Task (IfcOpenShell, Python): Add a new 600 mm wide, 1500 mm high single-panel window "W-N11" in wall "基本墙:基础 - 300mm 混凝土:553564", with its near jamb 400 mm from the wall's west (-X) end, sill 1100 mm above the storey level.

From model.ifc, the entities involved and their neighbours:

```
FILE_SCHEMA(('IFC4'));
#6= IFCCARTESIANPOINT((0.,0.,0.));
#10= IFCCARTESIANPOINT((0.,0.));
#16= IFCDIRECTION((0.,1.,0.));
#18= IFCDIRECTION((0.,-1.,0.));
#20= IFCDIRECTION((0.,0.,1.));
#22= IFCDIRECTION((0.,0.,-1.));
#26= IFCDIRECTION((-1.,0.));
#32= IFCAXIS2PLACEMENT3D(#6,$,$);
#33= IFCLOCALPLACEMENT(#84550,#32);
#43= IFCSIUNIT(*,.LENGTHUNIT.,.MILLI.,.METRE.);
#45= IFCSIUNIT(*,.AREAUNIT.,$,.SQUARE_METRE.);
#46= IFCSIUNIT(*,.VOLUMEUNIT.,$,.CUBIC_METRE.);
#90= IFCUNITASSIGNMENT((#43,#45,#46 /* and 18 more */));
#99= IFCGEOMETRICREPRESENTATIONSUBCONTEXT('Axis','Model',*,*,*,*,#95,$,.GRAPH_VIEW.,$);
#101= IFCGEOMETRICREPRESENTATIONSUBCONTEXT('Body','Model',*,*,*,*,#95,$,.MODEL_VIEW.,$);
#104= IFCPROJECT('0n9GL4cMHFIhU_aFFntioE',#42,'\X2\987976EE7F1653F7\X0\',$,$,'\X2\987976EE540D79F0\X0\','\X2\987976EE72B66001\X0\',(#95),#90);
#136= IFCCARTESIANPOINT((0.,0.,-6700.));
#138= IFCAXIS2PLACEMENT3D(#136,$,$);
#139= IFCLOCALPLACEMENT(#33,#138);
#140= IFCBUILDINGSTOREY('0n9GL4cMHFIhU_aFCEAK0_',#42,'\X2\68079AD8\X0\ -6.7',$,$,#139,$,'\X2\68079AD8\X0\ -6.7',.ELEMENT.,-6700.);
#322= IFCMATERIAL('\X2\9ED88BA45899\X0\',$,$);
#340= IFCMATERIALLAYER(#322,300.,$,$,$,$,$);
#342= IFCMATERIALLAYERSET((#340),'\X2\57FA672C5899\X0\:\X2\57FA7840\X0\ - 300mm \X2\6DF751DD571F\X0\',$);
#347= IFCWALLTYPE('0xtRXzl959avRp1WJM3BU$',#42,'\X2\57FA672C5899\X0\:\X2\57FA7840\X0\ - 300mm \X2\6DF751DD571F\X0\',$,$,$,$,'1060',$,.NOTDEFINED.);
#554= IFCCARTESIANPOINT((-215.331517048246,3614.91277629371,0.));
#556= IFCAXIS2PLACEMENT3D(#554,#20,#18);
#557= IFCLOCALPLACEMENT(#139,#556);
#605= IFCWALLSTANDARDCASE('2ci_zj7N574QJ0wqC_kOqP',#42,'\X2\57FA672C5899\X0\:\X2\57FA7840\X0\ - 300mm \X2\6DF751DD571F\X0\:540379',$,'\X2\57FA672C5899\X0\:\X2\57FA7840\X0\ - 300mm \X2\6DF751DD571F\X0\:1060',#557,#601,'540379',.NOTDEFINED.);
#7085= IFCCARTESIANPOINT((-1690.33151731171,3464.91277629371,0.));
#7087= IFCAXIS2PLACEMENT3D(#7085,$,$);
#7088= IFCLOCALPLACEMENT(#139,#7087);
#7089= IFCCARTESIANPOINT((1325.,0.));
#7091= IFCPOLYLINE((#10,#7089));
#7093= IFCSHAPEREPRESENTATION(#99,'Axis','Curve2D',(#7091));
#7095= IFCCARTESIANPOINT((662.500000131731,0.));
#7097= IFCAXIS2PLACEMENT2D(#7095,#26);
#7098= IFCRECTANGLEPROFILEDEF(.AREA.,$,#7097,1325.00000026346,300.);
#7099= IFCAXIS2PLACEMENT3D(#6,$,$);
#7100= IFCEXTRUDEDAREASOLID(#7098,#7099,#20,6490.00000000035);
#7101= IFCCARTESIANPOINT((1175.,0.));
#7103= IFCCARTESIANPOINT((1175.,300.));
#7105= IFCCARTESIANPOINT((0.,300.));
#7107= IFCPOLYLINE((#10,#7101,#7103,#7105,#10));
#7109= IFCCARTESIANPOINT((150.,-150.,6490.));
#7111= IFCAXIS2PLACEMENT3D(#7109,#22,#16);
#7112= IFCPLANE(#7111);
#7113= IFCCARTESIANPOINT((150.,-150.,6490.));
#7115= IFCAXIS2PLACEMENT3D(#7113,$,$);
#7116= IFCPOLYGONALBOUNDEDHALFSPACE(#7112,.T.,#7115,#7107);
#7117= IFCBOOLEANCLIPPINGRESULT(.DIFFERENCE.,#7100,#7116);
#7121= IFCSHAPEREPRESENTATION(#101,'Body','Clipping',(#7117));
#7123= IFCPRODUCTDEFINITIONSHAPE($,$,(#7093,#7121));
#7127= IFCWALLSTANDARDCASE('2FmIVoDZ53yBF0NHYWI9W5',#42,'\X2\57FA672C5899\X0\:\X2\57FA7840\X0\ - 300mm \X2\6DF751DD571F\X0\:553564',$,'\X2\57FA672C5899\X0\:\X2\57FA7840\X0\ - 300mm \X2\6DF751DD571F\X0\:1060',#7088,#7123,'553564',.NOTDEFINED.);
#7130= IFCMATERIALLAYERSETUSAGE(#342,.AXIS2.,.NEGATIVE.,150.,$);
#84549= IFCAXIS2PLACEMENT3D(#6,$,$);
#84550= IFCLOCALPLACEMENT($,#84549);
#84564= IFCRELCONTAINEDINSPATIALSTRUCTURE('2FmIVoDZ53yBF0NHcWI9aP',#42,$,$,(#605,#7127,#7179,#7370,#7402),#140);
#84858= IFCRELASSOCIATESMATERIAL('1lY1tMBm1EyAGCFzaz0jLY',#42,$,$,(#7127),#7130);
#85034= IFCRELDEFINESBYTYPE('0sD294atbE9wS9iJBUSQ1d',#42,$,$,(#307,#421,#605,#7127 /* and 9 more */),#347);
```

```python
import numpy as np
import ifcopenshell
import ifcopenshell.api.feature
import ifcopenshell.api.geometry
import ifcopenshell.api.root
import ifcopenshell.api.spatial
import ifcopenshell.geom
import ifcopenshell.util.element
import ifcopenshell.util.placement
import ifcopenshell.util.representation
import ifcopenshell.util.shape
import ifcopenshell.util.unit

model = ifcopenshell.open("model.ifc")
unit_scale = ifcopenshell.util.unit.calculate_unit_scale(model)
settings = ifcopenshell.geom.settings()


def volume(element):
    """Net volume in cubic metres, openings subtracted."""
    shape = ifcopenshell.geom.create_shape(settings, element)
    return ifcopenshell.util.shape.get_volume(shape.geometry)


wall = model.by_guid("2FmIVoDZ53yBF0NHYWI9W5")
storey = ifcopenshell.util.element.get_container(wall, ifc_class="IfcBuildingStorey")
context = ifcopenshell.util.representation.get_context(model, "Model", "Body", "MODEL_VIEW")
before = volume(wall)

width, height, from_end, sill = 0.6, 1.5, 0.4, 1.1  # metres

# The wall runs along its own X axis, and the end named is its -X end.
wall_shape = ifcopenshell.geom.create_shape(settings, wall)
x, y, z = ifcopenshell.util.shape.get_vertices(wall_shape.geometry).T
start = x.min() + from_end
face, thickness = float(y.min()), float(y.max() - y.min())
wall_matrix = ifcopenshell.util.placement.get_local_placement(wall.ObjectPlacement)
level = ifcopenshell.util.placement.get_local_placement(storey.ObjectPlacement)[2, 3]


def in_wall(x, y):
    """Placement at x, y metres in the wall's axes, at sill height."""
    matrix = wall_matrix.copy()
    matrix[:, 3] = wall_matrix @ np.array([x / unit_scale, y / unit_scale, 0.0, 1.0])
    matrix[2, 3] = level + sill / unit_scale
    return matrix


# Opening: a box that overshoots both wall faces by 50 mm.
opening = ifcopenshell.api.root.create_entity(model, ifc_class="IfcOpeningElement", predefined_type="OPENING")
box = ifcopenshell.api.geometry.add_wall_representation(
    model, context=context, length=width, height=height, thickness=thickness + 0.1
)
ifcopenshell.api.geometry.assign_representation(model, product=opening, representation=box)
ifcopenshell.api.geometry.edit_object_placement(model, product=opening, matrix=in_wall(start, face - 0.05), is_si=False)
ifcopenshell.api.feature.add_feature(model, feature=opening, element=wall)

window = ifcopenshell.api.root.create_entity(model, ifc_class="IfcWindow", name="W-N11", predefined_type="WINDOW")
window.OverallWidth, window.OverallHeight = width / unit_scale, height / unit_scale
window.PartitioningType = "SINGLE_PANEL"
body = ifcopenshell.api.geometry.add_window_representation(
    model,
    context=context,
    overall_width=window.OverallWidth,
    overall_height=window.OverallHeight,
    partition_type="SINGLE_PANEL",
)
ifcopenshell.api.geometry.assign_representation(model, product=window, representation=body)
ifcopenshell.api.spatial.assign_container(model, products=[window], relating_structure=storey)
ifcopenshell.api.feature.add_filling(model, opening=opening, element=window)

# Centre the window in the wall's thickness.
ifcopenshell.api.geometry.edit_object_placement(model, product=window, matrix=in_wall(start, face), is_si=False)
window_shape = ifcopenshell.geom.create_shape(settings, window)
depth = ifcopenshell.util.shape.get_vertices(window_shape.geometry)[:, 1]
offset = face + thickness / 2 - (depth.min() + depth.max()) / 2
ifcopenshell.api.geometry.edit_object_placement(model, product=window, matrix=in_wall(start, offset), is_si=False)

after = volume(wall)

print(f"wall volume {before:.3f} -> {after:.3f} m3")

model.write("model_v2.ifc")
```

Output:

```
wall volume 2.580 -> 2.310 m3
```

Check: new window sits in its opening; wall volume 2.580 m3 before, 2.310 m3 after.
